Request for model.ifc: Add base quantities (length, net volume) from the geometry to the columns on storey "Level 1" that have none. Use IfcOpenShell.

First a look at what the model holds.

```python
import ifcopenshell
import ifcopenshell.util.element
import ifcopenshell.util.unit

model = ifcopenshell.open("model.ifc")
print(model.schema)
for unit_type in ("LENGTHUNIT", "AREAUNIT", "VOLUMEUNIT"):
    print(unit_type, ifcopenshell.util.unit.calculate_unit_scale(model, unit_type))
storey = next(s for s in model.by_type("IfcBuildingStorey") if s.Name == "Level 1")
columns = [e for e in ifcopenshell.util.element.get_decomposition(storey) if e.is_a("IfcColumn")]
for e in sorted(columns, key=lambda e: e.id()):
    print(e.id(), e.is_a(), e.Name, list(ifcopenshell.util.element.get_psets(e, qtos_only=True)), sep=" | ")
```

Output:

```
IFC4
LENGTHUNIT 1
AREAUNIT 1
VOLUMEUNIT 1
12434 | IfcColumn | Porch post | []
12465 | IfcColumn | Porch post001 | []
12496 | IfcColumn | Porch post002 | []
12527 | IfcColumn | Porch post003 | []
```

```python
import ifcopenshell
import ifcopenshell.api.pset
import ifcopenshell.geom
import ifcopenshell.util.element
import ifcopenshell.util.shape
import ifcopenshell.util.unit

model = ifcopenshell.open("model.ifc")
unit_scale = ifcopenshell.util.unit.calculate_unit_scale(model)
volume_scale = ifcopenshell.util.unit.calculate_unit_scale(model, "VOLUMEUNIT")
settings = ifcopenshell.geom.settings()

storey = next(s for s in model.by_type("IfcBuildingStorey") if s.Name == "Level 1")
columns = [e for e in ifcopenshell.util.element.get_decomposition(storey) if e.is_a("IfcColumn")]

for e in sorted(columns, key=lambda e: e.id()):
    if ifcopenshell.util.element.get_psets(e, qtos_only=True, should_inherit=False):
        continue
    # Geometry comes back in metres, in the element's own axes.
    shape = ifcopenshell.geom.create_shape(settings, e)
    values = {
        "Length": ifcopenshell.util.shape.get_z(shape.geometry) / unit_scale,
        "NetVolume": ifcopenshell.util.shape.get_volume(shape.geometry) / volume_scale,
    }
    qto = ifcopenshell.api.pset.add_qto(model, product=e, name="Qto_ColumnBaseQuantities")
    ifcopenshell.api.pset.edit_qto(model, qto=qto, properties=values)
    print(e.id(), {k: round(v, 3) for k, v in values.items()})

model.write("model_edited.ifc")
```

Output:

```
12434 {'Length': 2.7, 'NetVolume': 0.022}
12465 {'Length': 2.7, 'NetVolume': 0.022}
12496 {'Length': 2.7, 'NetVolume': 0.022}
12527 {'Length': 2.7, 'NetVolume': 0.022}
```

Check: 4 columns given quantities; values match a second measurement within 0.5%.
